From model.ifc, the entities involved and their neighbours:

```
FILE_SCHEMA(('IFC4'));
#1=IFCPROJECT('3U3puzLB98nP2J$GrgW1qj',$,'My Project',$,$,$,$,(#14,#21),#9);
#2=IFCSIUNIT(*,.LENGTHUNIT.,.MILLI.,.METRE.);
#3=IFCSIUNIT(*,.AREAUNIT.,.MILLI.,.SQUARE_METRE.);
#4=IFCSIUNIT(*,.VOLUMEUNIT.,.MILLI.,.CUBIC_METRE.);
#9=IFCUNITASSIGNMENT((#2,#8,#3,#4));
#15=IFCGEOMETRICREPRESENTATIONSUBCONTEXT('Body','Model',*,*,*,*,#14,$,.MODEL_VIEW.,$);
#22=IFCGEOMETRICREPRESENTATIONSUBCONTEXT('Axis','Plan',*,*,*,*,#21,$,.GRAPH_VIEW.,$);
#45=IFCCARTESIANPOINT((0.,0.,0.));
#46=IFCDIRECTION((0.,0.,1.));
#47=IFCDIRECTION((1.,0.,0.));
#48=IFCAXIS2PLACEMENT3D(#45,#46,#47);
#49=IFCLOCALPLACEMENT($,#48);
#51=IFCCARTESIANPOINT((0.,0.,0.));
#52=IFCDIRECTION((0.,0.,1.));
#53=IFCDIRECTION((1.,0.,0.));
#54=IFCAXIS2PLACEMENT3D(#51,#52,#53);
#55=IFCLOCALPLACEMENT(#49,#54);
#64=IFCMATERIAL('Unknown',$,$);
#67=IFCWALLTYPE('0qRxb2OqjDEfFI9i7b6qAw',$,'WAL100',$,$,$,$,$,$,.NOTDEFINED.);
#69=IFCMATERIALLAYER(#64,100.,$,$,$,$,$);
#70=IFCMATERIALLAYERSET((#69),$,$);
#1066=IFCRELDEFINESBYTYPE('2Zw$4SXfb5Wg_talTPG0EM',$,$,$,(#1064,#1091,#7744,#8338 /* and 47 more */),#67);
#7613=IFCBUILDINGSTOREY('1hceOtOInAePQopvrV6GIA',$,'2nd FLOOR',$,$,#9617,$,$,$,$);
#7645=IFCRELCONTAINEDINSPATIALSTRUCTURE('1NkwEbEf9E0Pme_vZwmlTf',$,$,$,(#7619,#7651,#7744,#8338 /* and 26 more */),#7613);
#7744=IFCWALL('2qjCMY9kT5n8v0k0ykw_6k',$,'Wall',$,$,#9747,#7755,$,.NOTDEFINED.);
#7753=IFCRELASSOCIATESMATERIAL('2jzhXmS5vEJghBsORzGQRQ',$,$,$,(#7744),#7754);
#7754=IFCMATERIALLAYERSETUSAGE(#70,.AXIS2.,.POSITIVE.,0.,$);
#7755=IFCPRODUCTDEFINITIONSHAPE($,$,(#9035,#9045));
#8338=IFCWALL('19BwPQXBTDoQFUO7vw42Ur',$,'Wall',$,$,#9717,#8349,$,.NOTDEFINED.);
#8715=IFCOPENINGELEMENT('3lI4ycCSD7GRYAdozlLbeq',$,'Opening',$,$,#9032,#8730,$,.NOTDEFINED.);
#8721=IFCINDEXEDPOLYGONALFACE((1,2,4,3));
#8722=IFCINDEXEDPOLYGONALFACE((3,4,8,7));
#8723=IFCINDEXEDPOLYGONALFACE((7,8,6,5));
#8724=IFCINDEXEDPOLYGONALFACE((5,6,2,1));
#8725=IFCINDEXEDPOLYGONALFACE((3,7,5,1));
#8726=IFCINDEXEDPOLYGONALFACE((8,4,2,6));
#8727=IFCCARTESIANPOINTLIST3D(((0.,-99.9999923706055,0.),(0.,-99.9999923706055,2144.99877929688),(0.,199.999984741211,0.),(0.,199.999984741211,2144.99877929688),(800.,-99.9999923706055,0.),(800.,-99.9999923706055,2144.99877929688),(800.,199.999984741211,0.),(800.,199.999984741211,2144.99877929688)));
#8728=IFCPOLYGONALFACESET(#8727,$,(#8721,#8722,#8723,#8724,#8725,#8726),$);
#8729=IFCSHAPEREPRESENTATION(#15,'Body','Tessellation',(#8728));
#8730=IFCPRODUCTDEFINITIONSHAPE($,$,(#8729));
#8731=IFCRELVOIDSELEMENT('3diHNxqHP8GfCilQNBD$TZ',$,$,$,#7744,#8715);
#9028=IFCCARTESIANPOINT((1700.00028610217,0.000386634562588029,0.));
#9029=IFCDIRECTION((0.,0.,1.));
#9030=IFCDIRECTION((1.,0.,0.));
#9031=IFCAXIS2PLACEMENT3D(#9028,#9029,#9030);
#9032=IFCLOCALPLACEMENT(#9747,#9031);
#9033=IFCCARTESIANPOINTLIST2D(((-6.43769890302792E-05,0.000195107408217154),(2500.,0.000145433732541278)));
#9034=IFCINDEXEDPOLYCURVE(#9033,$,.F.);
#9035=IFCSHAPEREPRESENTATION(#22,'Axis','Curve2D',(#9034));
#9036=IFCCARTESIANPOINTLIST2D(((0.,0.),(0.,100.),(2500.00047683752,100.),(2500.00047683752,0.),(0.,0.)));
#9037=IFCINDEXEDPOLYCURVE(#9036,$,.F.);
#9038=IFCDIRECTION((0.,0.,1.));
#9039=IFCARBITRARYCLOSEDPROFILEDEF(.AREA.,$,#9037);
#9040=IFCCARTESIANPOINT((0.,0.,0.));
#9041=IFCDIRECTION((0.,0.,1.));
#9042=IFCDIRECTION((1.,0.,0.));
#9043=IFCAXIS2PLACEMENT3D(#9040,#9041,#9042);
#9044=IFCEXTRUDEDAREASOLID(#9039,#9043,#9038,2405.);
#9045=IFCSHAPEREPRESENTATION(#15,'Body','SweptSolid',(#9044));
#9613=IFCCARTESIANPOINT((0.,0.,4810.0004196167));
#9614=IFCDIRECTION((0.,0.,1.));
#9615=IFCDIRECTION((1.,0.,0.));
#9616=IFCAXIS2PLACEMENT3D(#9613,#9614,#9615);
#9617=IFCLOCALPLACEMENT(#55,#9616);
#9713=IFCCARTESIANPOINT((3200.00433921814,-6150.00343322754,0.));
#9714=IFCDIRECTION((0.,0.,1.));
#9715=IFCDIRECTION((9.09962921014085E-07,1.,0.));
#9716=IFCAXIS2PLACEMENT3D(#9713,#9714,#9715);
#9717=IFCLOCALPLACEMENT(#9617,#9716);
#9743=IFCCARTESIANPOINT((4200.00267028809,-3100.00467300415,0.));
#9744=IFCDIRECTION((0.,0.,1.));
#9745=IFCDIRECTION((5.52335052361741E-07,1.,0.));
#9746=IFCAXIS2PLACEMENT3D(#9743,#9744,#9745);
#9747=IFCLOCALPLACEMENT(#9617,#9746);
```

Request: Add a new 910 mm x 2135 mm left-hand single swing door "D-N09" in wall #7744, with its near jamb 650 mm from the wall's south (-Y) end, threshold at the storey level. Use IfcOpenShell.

```python
import numpy as np
import ifcopenshell
import ifcopenshell.api.feature
import ifcopenshell.api.geometry
import ifcopenshell.api.root
import ifcopenshell.api.spatial
import ifcopenshell.geom
import ifcopenshell.util.element
import ifcopenshell.util.placement
import ifcopenshell.util.representation
import ifcopenshell.util.shape
import ifcopenshell.util.unit

model = ifcopenshell.open("model.ifc")
unit_scale = ifcopenshell.util.unit.calculate_unit_scale(model)
settings = ifcopenshell.geom.settings()


def volume(element):
    """Net volume in cubic metres, openings subtracted."""
    shape = ifcopenshell.geom.create_shape(settings, element)
    return ifcopenshell.util.shape.get_volume(shape.geometry)


wall = model.by_guid("2qjCMY9kT5n8v0k0ykw_6k")
storey = ifcopenshell.util.element.get_container(wall, ifc_class="IfcBuildingStorey")
context = ifcopenshell.util.representation.get_context(model, "Model", "Body", "MODEL_VIEW")
before = volume(wall)

width, height, from_end, sill = 0.91, 2.135, 0.65, 0.0  # metres

# The wall runs along its own X axis, and the end named is its -X end.
wall_shape = ifcopenshell.geom.create_shape(settings, wall)
x, y, z = ifcopenshell.util.shape.get_vertices(wall_shape.geometry).T
start = x.min() + from_end
face, thickness = float(y.min()), float(y.max() - y.min())
wall_matrix = ifcopenshell.util.placement.get_local_placement(wall.ObjectPlacement)
level = ifcopenshell.util.placement.get_local_placement(storey.ObjectPlacement)[2, 3]


def in_wall(x, y):
    """Placement at x, y metres in the wall's axes, at sill height."""
    matrix = wall_matrix.copy()
    matrix[:, 3] = wall_matrix @ np.array([x / unit_scale, y / unit_scale, 0.0, 1.0])
    matrix[2, 3] = level + sill / unit_scale
    return matrix


# Opening: a box that overshoots both wall faces by 50 mm.
opening = ifcopenshell.api.root.create_entity(model, ifc_class="IfcOpeningElement", predefined_type="OPENING")
box = ifcopenshell.api.geometry.add_wall_representation(
    model, context=context, length=width, height=height, thickness=thickness + 0.1
)
ifcopenshell.api.geometry.assign_representation(model, product=opening, representation=box)
ifcopenshell.api.geometry.edit_object_placement(model, product=opening, matrix=in_wall(start, face - 0.05), is_si=False)
ifcopenshell.api.feature.add_feature(model, feature=opening, element=wall)

door = ifcopenshell.api.root.create_entity(model, ifc_class="IfcDoor", name="D-N09", predefined_type="DOOR")
door.OverallWidth, door.OverallHeight = width / unit_scale, height / unit_scale
door.OperationType = "SINGLE_SWING_LEFT"
body = ifcopenshell.api.geometry.add_door_representation(
    model,
    context=context,
    overall_width=door.OverallWidth,
    overall_height=door.OverallHeight,
    operation_type="SINGLE_SWING_LEFT",
    lining_properties={"LiningDepth": thickness / unit_scale, "ThresholdDepth": thickness / unit_scale},
)
ifcopenshell.api.geometry.assign_representation(model, product=door, representation=body)
ifcopenshell.api.spatial.assign_container(model, products=[door], relating_structure=storey)
ifcopenshell.api.feature.add_filling(model, opening=opening, element=door)

# The lining spans the wall, so the door starts at the wall face.
ifcopenshell.api.geometry.edit_object_placement(model, product=door, matrix=in_wall(start, face), is_si=False)

after = volume(wall)

print(f"wall volume {before:.3f} -> {after:.3f} m3")

model.write("model_rev.ifc")
```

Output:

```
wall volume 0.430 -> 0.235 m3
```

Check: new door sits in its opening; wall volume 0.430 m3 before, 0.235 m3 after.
